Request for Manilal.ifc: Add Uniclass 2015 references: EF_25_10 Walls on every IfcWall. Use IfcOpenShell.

First a look at what the model holds.

```python
import ifcopenshell

model = ifcopenshell.open("Manilal.ifc")
print(model.schema)
print("classifications:", [c.Name for c in model.by_type("IfcClassification")])
for ifc_class in ("IfcDoor", "IfcRoof", "IfcStair", "IfcWall", "IfcWindow"):
    print(ifc_class, len(model.by_type(ifc_class)))
```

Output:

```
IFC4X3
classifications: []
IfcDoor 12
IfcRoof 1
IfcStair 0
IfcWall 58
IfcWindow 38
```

```python
import ifcopenshell
import ifcopenshell.api.classification

model = ifcopenshell.open("Manilal.ifc")

system = ifcopenshell.api.classification.add_classification(model, classification="Uniclass 2015")

codes = {
    "IfcWall": ("EF_25_10", "Walls"),
}
for ifc_class, (code, name) in codes.items():
    products = model.by_type(ifc_class)
    ifcopenshell.api.classification.add_reference(
        model, products=products, classification=system, identification=code, name=name
    )
    print(code, len(products))

model.write("Manilal_edited.ifc")
```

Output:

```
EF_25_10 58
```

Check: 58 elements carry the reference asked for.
